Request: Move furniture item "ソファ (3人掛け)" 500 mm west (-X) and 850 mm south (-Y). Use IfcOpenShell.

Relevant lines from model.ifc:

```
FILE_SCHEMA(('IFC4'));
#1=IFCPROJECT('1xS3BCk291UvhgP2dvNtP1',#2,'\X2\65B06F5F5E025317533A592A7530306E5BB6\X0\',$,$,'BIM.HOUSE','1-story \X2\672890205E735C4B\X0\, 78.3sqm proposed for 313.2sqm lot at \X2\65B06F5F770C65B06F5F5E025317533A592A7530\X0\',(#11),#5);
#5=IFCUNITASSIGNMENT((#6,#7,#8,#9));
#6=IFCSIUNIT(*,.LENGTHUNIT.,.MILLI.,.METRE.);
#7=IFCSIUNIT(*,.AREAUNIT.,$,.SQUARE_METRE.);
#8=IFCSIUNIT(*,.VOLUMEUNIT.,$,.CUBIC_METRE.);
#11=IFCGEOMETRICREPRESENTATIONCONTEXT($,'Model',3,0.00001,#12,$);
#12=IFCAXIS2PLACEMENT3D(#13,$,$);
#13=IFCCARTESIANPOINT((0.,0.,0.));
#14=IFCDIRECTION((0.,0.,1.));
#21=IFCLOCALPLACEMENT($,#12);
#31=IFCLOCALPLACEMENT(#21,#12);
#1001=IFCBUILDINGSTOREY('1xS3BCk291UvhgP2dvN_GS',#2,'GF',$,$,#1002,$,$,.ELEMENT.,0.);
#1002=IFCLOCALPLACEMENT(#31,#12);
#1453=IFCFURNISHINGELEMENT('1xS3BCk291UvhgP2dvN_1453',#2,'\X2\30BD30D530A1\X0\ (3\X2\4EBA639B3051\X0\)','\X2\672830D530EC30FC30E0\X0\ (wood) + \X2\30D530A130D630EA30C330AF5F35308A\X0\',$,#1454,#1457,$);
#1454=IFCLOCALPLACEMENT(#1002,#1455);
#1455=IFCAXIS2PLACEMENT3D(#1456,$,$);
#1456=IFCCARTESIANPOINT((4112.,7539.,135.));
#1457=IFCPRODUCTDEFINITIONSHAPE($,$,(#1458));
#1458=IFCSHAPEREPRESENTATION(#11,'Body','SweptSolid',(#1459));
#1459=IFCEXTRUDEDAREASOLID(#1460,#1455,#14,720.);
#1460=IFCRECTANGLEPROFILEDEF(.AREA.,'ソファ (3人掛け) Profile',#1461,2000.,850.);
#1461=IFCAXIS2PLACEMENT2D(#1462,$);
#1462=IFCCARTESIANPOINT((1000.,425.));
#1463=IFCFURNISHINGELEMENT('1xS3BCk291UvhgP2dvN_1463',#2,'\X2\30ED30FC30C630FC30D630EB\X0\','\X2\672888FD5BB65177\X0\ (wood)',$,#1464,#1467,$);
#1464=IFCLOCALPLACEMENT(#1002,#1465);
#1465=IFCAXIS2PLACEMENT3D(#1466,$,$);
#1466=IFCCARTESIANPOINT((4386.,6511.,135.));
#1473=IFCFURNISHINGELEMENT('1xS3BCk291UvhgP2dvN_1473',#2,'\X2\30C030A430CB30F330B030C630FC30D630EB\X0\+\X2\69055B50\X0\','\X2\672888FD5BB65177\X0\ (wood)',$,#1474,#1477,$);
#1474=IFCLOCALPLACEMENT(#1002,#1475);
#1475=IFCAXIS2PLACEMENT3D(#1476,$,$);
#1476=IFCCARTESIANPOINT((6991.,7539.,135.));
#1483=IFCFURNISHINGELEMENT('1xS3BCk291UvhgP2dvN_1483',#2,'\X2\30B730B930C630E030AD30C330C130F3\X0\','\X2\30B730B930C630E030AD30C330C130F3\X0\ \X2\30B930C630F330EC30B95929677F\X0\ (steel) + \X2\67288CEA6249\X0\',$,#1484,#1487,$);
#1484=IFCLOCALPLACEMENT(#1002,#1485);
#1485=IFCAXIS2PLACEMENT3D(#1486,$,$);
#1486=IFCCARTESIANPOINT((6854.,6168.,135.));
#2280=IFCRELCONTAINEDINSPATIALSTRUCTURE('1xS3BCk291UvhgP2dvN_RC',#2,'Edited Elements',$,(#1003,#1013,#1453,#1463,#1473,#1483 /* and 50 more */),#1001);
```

```python
import ifcopenshell
import ifcopenshell.api.geometry
import ifcopenshell.util.placement

model = ifcopenshell.open("model.ifc")

item = model.by_id(1453)
matrix = ifcopenshell.util.placement.get_local_placement(item.ObjectPlacement)
matrix[0, 3] -= 500.0
matrix[1, 3] -= 850.0
ifcopenshell.api.geometry.edit_object_placement(model, product=item, matrix=matrix, is_si=False)

print(ifcopenshell.util.placement.get_local_placement(item.ObjectPlacement).round(3) + 0.0)

model.write("model_updated.ifc")
```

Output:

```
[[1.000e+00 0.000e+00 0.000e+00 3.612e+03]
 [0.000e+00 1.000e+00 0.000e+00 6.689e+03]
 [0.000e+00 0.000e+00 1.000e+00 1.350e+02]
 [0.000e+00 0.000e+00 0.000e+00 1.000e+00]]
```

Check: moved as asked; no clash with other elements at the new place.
